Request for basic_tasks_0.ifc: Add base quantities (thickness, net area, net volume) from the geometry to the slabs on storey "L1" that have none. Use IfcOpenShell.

First a look at what the model holds.

```python
import ifcopenshell
import ifcopenshell.util.element
import ifcopenshell.util.unit

model = ifcopenshell.open("basic_tasks_0.ifc")
print(model.schema)
for unit_type in ("LENGTHUNIT", "AREAUNIT", "VOLUMEUNIT"):
    print(unit_type, ifcopenshell.util.unit.calculate_unit_scale(model, unit_type))
storey = next(s for s in model.by_type("IfcBuildingStorey") if s.Name == "L1")
slabs = [e for e in ifcopenshell.util.element.get_decomposition(storey) if e.is_a("IfcSlab")]
for e in sorted(slabs, key=lambda e: e.id()):
    print(e.id(), e.is_a(), e.Name, list(ifcopenshell.util.element.get_psets(e, qtos_only=True)), sep=" | ")
```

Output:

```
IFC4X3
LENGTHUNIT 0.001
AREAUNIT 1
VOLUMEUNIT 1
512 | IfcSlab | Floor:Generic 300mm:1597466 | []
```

```python
import ifcopenshell
import ifcopenshell.api.pset
import ifcopenshell.geom
import ifcopenshell.util.element
import ifcopenshell.util.shape
import ifcopenshell.util.unit

model = ifcopenshell.open("basic_tasks_0.ifc")
unit_scale = ifcopenshell.util.unit.calculate_unit_scale(model)
area_scale = ifcopenshell.util.unit.calculate_unit_scale(model, "AREAUNIT")
volume_scale = ifcopenshell.util.unit.calculate_unit_scale(model, "VOLUMEUNIT")
settings = ifcopenshell.geom.settings()

storey = next(s for s in model.by_type("IfcBuildingStorey") if s.Name == "L1")
slabs = [e for e in ifcopenshell.util.element.get_decomposition(storey) if e.is_a("IfcSlab")]

for e in sorted(slabs, key=lambda e: e.id()):
    if ifcopenshell.util.element.get_psets(e, qtos_only=True, should_inherit=False):
        continue
    # Geometry comes back in metres, in the element's own axes.
    shape = ifcopenshell.geom.create_shape(settings, e)
    values = {
        "Width": ifcopenshell.util.shape.get_z(shape.geometry) / unit_scale,
        "NetArea": ifcopenshell.util.shape.get_footprint_area(shape.geometry) / area_scale,
        "NetVolume": ifcopenshell.util.shape.get_volume(shape.geometry) / volume_scale,
    }
    qto = ifcopenshell.api.pset.add_qto(model, product=e, name="Qto_SlabBaseQuantities")
    ifcopenshell.api.pset.edit_qto(model, qto=qto, properties=values)
    print(e.id(), {k: round(v, 3) for k, v in values.items()})

model.write("basic_tasks_0_v2.ifc")
```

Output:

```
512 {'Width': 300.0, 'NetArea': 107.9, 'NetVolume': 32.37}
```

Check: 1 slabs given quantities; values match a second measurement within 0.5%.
